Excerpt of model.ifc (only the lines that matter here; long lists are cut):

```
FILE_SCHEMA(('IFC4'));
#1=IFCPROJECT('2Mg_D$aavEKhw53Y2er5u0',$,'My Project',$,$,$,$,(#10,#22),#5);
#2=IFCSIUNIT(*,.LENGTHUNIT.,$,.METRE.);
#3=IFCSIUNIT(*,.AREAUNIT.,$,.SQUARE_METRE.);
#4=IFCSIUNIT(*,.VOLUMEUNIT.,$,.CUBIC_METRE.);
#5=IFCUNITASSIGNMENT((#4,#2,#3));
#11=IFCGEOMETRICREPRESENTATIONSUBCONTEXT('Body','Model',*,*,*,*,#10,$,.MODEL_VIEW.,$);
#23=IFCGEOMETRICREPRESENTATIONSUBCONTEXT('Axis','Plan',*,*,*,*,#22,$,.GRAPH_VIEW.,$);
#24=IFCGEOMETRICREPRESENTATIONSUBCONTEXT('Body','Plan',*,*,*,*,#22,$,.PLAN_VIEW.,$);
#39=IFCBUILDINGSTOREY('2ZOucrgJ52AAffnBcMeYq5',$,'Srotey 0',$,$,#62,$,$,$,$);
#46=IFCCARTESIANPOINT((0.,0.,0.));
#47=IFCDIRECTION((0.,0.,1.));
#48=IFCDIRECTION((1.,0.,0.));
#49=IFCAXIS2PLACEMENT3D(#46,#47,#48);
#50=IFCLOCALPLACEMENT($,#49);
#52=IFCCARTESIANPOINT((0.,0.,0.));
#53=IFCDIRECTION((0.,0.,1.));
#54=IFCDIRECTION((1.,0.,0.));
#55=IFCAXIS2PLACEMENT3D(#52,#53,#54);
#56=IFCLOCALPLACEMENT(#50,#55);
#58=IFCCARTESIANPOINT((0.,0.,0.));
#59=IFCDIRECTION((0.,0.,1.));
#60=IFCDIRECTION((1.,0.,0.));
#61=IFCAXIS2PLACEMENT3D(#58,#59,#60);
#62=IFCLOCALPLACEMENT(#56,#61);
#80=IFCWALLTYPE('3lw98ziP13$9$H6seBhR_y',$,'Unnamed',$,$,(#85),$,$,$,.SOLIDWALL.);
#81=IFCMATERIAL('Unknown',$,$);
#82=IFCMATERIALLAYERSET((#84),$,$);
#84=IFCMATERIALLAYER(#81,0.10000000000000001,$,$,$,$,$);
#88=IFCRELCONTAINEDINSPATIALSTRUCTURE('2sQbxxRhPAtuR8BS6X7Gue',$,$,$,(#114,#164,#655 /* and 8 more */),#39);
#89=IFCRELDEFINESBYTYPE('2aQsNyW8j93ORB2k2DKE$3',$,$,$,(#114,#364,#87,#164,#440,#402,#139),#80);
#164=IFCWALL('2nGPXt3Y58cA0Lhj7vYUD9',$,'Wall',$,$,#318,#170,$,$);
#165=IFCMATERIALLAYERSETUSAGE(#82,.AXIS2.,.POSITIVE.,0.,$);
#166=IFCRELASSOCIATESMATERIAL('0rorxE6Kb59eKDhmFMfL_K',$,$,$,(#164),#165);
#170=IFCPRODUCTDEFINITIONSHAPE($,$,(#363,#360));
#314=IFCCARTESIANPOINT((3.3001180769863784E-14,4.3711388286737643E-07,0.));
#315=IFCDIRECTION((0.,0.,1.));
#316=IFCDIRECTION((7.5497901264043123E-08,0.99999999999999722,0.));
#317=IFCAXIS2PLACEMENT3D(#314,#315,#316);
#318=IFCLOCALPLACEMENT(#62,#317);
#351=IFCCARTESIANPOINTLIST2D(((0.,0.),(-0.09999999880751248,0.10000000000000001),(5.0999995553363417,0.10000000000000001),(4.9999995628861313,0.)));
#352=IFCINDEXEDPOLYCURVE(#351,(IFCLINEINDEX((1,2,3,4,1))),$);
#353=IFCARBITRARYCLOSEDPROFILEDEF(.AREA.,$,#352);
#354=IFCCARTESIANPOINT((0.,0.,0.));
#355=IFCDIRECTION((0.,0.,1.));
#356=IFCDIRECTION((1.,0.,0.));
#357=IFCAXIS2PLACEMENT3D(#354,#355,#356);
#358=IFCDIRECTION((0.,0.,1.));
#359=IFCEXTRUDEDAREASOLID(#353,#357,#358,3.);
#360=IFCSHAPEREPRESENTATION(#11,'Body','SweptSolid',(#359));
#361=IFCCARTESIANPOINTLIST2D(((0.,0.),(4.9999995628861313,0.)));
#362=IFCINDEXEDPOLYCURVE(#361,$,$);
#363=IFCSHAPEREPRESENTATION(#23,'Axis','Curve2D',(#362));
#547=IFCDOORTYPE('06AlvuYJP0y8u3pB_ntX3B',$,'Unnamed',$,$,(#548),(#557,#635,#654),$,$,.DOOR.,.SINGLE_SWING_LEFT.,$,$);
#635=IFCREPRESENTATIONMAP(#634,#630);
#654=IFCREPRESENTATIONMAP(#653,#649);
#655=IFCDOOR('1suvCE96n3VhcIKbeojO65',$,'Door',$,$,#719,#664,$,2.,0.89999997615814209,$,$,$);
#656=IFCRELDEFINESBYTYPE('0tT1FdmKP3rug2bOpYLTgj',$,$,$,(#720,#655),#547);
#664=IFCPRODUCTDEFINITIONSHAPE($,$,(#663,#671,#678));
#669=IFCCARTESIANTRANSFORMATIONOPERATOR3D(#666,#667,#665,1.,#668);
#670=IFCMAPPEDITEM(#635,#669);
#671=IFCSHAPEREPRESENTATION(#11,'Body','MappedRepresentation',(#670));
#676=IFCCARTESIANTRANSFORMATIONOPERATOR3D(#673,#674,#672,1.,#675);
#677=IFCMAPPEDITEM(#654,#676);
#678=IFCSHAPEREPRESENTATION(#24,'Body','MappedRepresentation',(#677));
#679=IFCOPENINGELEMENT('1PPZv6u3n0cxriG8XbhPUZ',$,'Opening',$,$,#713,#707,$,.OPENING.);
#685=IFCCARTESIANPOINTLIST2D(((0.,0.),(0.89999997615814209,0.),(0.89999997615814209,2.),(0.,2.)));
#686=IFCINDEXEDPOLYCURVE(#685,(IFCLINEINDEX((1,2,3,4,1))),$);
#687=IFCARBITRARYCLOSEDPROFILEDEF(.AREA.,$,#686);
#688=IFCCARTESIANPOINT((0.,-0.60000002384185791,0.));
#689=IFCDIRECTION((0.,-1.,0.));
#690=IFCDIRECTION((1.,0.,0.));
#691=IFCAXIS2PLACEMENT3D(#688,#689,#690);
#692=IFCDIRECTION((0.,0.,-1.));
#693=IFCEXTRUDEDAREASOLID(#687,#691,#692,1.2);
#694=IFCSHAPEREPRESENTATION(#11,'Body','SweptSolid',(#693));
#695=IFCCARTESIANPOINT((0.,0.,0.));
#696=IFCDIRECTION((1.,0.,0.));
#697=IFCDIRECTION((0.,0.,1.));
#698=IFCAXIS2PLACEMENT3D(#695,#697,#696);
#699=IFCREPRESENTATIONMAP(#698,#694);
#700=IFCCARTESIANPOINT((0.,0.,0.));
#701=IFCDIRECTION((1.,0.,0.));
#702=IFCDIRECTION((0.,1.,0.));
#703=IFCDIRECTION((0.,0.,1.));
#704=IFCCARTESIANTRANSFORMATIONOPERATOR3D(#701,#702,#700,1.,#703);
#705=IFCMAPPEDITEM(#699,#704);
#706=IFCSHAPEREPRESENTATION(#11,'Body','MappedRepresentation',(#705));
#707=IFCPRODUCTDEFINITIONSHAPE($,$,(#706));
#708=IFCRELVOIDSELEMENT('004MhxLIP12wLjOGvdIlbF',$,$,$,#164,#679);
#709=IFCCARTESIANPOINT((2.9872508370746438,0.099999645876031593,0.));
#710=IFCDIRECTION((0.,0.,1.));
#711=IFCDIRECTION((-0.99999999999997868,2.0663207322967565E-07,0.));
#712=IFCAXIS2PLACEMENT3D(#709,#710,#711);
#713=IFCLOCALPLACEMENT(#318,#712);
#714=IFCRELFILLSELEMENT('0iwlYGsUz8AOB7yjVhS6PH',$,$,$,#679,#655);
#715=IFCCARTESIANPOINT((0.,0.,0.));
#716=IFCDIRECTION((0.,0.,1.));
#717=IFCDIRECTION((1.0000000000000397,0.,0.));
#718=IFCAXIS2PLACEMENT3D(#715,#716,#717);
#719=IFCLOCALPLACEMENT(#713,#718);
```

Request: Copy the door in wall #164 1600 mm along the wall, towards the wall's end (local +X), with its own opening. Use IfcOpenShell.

```python
import ifcopenshell
import ifcopenshell.api.feature
import ifcopenshell.api.geometry
import ifcopenshell.api.root
import ifcopenshell.geom
import ifcopenshell.util.element
import ifcopenshell.util.placement
import ifcopenshell.util.shape
import ifcopenshell.util.unit

model = ifcopenshell.open("model.ifc")
unit_scale = ifcopenshell.util.unit.calculate_unit_scale(model)
settings = ifcopenshell.geom.settings()


def volume(element):
    """Net volume in cubic metres, openings subtracted."""
    shape = ifcopenshell.geom.create_shape(settings, element)
    return ifcopenshell.util.shape.get_volume(shape.geometry)


door = model.by_id(655)
opening = door.FillsVoids[0].RelatingOpeningElement
wall = opening.VoidsElements[0].RelatingBuildingElement
before = volume(wall)
shift = ifcopenshell.util.placement.get_local_placement(wall.ObjectPlacement)[:3, 0] * 1.6 / unit_scale

# copy_class copies the void relationship, type, container and properties, but no geometry.
new_opening = ifcopenshell.api.root.copy_class(model, product=opening)
new_opening.Representation = ifcopenshell.util.element.copy_deep(
    model, opening.Representation, exclude=["IfcGeometricRepresentationContext", "IfcRepresentationMap"]
)
new_door = ifcopenshell.api.root.copy_class(model, product=door)
new_door.Representation = ifcopenshell.util.element.copy_deep(
    model, door.Representation, exclude=["IfcGeometricRepresentationContext", "IfcRepresentationMap"]
)
ifcopenshell.api.feature.add_filling(model, opening=new_opening, element=new_door)

for old, new in ((opening, new_opening), (door, new_door)):
    matrix = ifcopenshell.util.placement.get_local_placement(old.ObjectPlacement)
    matrix[:3, 3] += shift
    ifcopenshell.api.geometry.edit_object_placement(model, product=new, matrix=matrix, is_si=False)

after = volume(wall)

print(f"wall volume {before:.3f} -> {after:.3f} m3")

model.write("model_edited.ifc")
```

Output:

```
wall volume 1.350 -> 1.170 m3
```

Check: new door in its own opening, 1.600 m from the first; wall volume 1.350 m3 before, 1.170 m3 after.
